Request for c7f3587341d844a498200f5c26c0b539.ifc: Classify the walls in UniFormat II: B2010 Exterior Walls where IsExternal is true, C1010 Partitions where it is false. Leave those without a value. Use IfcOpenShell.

First a look at what the model holds.

```python
import ifcopenshell
import ifcopenshell.util.element

model = ifcopenshell.open("c7f3587341d844a498200f5c26c0b539.ifc")
print(model.schema)
print("classifications:", [c.Name for c in model.by_type("IfcClassification")])
values = [ifcopenshell.util.element.get_pset(e, "Pset_WallCommon", "IsExternal") for e in model.by_type("IfcWall")]
for value in (True, False, None):
    print("IsExternal", value, values.count(value))
```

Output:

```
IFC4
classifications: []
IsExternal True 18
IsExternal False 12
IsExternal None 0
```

```python
import ifcopenshell
import ifcopenshell.api.classification
import ifcopenshell.util.element

model = ifcopenshell.open("c7f3587341d844a498200f5c26c0b539.ifc")

system = ifcopenshell.api.classification.add_classification(model, classification="UniFormat II")

walls = model.by_type("IfcWall")
external = {e: ifcopenshell.util.element.get_pset(e, "Pset_WallCommon", "IsExternal") for e in walls}
for flag, code, name in ((True, "B2010", "Exterior Walls"), (False, "C1010", "Partitions")):
    products = [e for e in walls if external[e] is flag]
    ifcopenshell.api.classification.add_reference(
        model, products=products, classification=system, identification=code, name=name
    )
    print(code, len(products))

model.write("c7f3587341d844a498200f5c26c0b539_edited.ifc")
```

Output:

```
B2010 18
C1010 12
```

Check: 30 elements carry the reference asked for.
